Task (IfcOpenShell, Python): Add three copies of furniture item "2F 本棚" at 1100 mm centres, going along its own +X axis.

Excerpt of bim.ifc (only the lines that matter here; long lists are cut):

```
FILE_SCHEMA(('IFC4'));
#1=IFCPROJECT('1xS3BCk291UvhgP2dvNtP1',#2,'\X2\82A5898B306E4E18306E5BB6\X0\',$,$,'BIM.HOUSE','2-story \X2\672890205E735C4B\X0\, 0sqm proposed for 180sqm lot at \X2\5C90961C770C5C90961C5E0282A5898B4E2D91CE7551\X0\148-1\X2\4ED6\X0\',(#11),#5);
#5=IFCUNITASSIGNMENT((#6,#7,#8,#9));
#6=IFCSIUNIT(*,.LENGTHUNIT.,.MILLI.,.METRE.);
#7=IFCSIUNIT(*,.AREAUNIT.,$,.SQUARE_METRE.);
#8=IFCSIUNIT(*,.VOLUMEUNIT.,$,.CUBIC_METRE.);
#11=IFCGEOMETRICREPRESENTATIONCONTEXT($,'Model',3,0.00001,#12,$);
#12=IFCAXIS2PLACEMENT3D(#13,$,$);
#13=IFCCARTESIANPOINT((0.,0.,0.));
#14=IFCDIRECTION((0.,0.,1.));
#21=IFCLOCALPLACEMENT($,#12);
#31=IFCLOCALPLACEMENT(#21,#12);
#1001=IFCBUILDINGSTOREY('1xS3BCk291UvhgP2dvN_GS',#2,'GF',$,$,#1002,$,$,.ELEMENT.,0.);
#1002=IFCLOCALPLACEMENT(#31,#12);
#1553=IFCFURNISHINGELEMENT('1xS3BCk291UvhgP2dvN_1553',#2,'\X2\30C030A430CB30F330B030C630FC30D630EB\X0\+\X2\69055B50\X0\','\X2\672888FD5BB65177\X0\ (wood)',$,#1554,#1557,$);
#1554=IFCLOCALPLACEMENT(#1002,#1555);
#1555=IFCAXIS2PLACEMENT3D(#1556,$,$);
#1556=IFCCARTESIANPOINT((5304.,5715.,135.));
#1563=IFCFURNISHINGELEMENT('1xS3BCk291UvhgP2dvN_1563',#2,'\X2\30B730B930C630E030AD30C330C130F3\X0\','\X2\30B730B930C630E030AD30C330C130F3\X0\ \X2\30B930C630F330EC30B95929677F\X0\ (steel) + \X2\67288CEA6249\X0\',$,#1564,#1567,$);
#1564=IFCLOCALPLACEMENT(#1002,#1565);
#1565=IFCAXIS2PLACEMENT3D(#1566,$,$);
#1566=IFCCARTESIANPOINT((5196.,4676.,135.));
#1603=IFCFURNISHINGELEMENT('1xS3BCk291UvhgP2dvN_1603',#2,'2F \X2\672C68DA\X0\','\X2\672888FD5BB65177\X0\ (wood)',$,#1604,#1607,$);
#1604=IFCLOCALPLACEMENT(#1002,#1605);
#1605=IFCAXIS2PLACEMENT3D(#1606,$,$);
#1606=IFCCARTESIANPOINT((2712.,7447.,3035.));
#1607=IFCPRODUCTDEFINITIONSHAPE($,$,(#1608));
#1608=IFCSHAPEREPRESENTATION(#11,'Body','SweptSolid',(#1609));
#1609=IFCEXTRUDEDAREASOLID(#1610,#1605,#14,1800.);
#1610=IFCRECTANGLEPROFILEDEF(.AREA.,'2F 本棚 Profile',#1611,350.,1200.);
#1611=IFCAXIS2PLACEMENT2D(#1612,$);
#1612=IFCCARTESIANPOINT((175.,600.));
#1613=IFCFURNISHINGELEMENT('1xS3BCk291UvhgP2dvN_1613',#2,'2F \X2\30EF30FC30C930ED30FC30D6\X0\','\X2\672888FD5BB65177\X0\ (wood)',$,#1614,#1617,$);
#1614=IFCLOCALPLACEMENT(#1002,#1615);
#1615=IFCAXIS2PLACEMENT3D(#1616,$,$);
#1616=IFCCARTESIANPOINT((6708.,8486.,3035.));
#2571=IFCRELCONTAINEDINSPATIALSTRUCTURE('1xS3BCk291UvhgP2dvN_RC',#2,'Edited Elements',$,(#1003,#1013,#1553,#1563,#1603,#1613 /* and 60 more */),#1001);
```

```python
import ifcopenshell
import ifcopenshell.api.geometry
import ifcopenshell.api.root
import ifcopenshell.util.element
import ifcopenshell.util.placement

model = ifcopenshell.open("bim.ifc")


def reuse_history(source, copy):
    """copy_class also copies each property set's owner history, people and application; keep the originals."""
    for rel in copy.IsDefinedBy:
        if rel.is_a("IfcRelDefinesByProperties") and (history := rel.RelatingPropertyDefinition.OwnerHistory):
            rel.RelatingPropertyDefinition.OwnerHistory = source.OwnerHistory
            ifcopenshell.util.element.remove_deep2(model, history)


source = model.by_guid("1xS3BCk291UvhgP2dvN_1603")
base = ifcopenshell.util.placement.get_local_placement(source.ObjectPlacement)
step = base[:3, 0] * 1100.0

for i in range(1, 4):
    copy = ifcopenshell.api.root.copy_class(model, product=source)
    copy.Representation = ifcopenshell.util.element.copy_deep(
        model, source.Representation, exclude=["IfcGeometricRepresentationContext", "IfcRepresentationMap"]
    )
    reuse_history(source, copy)
    matrix = base.copy()
    matrix[:3, 3] += i * step
    print("added at", matrix[:3, 3].round(3) + 0.0)
    ifcopenshell.api.geometry.edit_object_placement(model, product=copy, matrix=matrix, is_si=False)

model.write("bim_updated.ifc")
```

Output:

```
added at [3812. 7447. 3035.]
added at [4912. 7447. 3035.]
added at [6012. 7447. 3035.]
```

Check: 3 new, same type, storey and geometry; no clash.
